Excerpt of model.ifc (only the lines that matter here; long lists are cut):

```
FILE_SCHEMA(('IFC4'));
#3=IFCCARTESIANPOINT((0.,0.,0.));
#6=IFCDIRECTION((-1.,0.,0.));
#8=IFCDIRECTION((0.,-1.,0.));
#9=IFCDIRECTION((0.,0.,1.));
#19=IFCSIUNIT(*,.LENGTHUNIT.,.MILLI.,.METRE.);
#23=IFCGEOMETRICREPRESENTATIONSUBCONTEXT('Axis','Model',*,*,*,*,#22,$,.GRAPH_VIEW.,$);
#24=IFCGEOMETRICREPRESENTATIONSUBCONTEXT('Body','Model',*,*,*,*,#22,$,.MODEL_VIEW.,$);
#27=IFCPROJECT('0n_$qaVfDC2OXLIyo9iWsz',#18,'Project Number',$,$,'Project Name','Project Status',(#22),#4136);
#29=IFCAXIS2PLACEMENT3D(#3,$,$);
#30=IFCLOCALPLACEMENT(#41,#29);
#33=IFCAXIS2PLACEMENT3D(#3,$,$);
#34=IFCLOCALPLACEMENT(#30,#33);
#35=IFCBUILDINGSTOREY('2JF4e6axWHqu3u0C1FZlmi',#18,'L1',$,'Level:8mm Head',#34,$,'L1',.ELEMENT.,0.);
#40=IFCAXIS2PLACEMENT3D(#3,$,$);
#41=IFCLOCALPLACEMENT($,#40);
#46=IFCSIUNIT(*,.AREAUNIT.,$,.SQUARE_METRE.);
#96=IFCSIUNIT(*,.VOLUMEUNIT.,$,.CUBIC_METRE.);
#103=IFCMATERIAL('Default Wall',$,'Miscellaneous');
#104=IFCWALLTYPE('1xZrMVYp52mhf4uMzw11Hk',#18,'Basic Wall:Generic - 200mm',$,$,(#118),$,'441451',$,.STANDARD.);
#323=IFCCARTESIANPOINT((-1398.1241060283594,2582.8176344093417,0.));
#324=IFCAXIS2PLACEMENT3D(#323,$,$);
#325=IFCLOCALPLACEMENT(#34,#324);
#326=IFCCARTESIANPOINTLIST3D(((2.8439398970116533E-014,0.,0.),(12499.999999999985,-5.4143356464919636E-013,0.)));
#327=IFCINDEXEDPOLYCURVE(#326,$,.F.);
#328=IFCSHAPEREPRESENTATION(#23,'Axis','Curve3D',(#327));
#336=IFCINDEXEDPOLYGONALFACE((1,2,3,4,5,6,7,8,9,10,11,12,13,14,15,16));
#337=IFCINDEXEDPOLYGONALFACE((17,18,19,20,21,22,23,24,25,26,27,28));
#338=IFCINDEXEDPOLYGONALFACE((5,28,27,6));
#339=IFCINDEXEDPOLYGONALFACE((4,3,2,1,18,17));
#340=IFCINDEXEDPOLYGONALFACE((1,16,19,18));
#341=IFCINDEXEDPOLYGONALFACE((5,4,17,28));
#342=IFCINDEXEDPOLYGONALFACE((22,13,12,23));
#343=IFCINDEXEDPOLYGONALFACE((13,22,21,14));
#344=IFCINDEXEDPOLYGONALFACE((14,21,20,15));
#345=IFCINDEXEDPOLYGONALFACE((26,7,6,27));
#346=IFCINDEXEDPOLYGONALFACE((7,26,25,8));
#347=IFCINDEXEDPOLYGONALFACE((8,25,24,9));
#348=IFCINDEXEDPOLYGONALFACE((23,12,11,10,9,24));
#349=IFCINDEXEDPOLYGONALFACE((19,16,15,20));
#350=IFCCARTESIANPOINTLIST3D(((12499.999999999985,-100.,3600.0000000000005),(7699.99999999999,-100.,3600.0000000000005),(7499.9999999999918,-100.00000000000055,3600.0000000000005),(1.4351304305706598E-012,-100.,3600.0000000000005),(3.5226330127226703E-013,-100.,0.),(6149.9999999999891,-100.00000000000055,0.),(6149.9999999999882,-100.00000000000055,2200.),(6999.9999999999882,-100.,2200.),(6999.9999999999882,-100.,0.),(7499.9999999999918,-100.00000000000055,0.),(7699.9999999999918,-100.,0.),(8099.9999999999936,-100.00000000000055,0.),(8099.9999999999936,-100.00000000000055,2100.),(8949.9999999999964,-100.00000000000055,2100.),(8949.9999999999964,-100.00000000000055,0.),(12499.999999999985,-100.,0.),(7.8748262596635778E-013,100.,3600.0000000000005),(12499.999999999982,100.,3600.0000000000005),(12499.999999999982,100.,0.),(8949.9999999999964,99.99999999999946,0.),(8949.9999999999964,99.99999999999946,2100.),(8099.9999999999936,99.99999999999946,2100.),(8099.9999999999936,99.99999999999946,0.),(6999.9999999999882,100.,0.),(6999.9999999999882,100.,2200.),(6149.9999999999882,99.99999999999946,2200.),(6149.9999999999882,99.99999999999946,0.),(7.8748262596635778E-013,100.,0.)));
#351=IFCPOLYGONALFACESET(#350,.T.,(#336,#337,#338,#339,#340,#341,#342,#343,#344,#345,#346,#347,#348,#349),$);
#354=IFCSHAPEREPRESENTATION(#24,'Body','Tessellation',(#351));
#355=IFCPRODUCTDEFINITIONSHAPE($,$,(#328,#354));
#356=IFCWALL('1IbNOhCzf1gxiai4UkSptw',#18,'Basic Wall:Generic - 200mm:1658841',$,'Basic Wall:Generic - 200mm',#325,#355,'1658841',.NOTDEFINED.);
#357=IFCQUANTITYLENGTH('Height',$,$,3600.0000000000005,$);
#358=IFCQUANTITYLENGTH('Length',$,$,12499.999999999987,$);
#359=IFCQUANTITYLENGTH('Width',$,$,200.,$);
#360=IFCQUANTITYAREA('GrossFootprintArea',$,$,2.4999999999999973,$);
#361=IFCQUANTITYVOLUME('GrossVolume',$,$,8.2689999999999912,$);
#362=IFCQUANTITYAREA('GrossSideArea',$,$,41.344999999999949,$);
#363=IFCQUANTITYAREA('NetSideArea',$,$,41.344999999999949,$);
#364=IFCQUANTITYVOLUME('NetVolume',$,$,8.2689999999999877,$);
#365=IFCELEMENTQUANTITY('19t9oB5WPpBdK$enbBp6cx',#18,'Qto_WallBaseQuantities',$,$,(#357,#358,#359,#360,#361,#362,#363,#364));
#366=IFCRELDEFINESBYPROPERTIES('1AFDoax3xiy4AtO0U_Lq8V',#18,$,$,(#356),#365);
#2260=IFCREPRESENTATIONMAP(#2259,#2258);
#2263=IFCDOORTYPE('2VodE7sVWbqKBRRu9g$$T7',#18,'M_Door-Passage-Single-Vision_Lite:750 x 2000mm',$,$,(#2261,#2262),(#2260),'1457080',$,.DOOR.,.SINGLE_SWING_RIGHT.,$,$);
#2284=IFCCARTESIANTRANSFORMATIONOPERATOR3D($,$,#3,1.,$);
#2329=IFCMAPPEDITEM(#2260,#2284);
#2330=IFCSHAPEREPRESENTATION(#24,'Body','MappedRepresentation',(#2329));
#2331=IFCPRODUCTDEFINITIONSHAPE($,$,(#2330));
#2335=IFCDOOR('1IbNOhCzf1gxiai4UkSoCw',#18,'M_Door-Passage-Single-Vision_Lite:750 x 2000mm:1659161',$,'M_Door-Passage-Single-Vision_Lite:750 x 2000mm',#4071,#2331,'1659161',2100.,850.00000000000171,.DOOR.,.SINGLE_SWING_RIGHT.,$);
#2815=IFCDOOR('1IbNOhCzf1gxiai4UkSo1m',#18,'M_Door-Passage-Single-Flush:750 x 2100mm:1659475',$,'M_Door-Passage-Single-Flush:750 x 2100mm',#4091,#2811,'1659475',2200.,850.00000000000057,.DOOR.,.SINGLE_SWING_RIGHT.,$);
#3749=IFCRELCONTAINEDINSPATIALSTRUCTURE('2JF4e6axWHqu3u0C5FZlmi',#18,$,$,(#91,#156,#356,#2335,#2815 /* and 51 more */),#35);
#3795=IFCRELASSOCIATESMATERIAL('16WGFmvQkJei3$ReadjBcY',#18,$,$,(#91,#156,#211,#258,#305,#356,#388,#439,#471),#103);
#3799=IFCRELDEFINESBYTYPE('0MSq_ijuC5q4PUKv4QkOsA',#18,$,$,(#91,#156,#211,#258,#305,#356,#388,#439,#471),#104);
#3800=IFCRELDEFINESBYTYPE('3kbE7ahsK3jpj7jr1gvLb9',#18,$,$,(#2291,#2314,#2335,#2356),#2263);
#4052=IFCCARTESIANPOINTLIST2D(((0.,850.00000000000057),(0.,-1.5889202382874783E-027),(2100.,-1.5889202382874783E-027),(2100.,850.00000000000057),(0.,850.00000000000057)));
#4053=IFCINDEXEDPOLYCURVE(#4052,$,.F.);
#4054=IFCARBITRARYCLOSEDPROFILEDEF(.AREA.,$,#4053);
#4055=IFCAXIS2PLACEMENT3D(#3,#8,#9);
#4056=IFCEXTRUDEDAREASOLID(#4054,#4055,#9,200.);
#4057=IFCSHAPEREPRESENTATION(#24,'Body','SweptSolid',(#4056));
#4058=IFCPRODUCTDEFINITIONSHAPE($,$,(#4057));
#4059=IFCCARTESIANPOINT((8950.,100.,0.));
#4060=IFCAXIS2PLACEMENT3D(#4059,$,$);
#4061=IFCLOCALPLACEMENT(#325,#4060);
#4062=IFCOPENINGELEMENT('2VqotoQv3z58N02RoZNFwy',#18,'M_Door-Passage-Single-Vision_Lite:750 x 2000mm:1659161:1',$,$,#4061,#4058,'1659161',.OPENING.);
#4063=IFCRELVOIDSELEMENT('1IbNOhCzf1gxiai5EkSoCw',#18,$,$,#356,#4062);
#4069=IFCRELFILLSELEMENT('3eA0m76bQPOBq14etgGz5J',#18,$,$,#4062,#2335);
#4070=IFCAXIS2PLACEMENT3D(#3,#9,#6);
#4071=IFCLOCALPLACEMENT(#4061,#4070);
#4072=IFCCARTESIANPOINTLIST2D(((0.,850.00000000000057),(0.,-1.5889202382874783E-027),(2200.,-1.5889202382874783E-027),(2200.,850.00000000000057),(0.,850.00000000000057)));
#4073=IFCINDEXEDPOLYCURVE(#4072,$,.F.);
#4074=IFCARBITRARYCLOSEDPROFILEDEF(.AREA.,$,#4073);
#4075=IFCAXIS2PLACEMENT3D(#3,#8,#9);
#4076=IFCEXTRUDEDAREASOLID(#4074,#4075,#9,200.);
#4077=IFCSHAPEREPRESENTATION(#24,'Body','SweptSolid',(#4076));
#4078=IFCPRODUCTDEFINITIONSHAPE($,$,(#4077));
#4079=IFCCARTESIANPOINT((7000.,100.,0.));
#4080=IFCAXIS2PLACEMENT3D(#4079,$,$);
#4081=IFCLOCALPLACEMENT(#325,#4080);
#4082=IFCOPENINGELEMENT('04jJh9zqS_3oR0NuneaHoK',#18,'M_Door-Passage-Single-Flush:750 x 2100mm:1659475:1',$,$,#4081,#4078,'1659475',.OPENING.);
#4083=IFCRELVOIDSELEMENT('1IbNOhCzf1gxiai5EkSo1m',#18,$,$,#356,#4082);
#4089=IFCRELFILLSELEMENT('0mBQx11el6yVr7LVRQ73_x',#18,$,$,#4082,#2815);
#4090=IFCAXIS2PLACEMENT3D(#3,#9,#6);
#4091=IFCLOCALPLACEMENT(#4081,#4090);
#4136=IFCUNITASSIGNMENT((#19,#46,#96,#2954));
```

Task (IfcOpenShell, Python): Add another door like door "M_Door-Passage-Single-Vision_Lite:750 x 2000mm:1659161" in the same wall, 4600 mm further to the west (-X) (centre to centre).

```python
import ifcopenshell
import ifcopenshell.api.feature
import ifcopenshell.api.geometry
import ifcopenshell.api.pset
import ifcopenshell.api.root
import ifcopenshell.geom
import ifcopenshell.util.element
import ifcopenshell.util.placement
import ifcopenshell.util.shape
import ifcopenshell.util.unit

model = ifcopenshell.open("model.ifc")
unit_scale = ifcopenshell.util.unit.calculate_unit_scale(model)
area_scale = ifcopenshell.util.unit.calculate_unit_scale(model, "AREAUNIT")
volume_scale = ifcopenshell.util.unit.calculate_unit_scale(model, "VOLUMEUNIT")
settings = ifcopenshell.geom.settings()


def volume(element):
    """Net volume in cubic metres, openings subtracted."""
    shape = ifcopenshell.geom.create_shape(settings, element)
    return ifcopenshell.util.shape.get_volume(shape.geometry)


def reuse_history(source, copy):
    """copy_class also copies each property set's owner history, people and application; keep the originals."""
    for rel in copy.IsDefinedBy:
        if rel.is_a("IfcRelDefinesByProperties") and (history := rel.RelatingPropertyDefinition.OwnerHistory):
            rel.RelatingPropertyDefinition.OwnerHistory = source.OwnerHistory
            ifcopenshell.util.element.remove_deep2(model, history)


door = model.by_id(2335)
opening = door.FillsVoids[0].RelatingOpeningElement
wall = opening.VoidsElements[0].RelatingBuildingElement
before = volume(wall)
shift = ifcopenshell.util.placement.get_local_placement(wall.ObjectPlacement)[:3, 0] * -4.6 / unit_scale

# copy_class copies the void relationship, type, container and properties, but no geometry.
new_opening = ifcopenshell.api.root.copy_class(model, product=opening)
new_opening.Representation = ifcopenshell.util.element.copy_deep(
    model, opening.Representation, exclude=["IfcGeometricRepresentationContext", "IfcRepresentationMap"]
)
new_opening.Name = "M_Door-Passage-Single-Vision_Lite:750 x 2000mm"
new_opening.Tag = None
reuse_history(opening, new_opening)
new_door = ifcopenshell.api.root.copy_class(model, product=door)
new_door.Representation = ifcopenshell.util.element.copy_deep(
    model, door.Representation, exclude=["IfcGeometricRepresentationContext", "IfcRepresentationMap"]
)
new_door.Name = "M_Door-Passage-Single-Vision_Lite:750 x 2000mm"
new_door.Tag = None
reuse_history(door, new_door)
ifcopenshell.api.feature.add_filling(model, opening=new_opening, element=new_door)

for old, new in ((opening, new_opening), (door, new_door)):
    matrix = ifcopenshell.util.placement.get_local_placement(old.ObjectPlacement)
    matrix[:3, 3] += shift
    ifcopenshell.api.geometry.edit_object_placement(model, product=new, matrix=matrix, is_si=False)

after = volume(wall)
thickness = 0.2  # wall thickness in metres

# Update the wall's stored quantities.
qto = model.by_id(ifcopenshell.util.element.get_pset(wall, "Qto_WallBaseQuantities", should_inherit=False)["id"])
ifcopenshell.api.pset.edit_qto(model, qto=qto, properties={
    "NetSideArea": after / thickness / area_scale,
    "NetVolume": after / volume_scale,
})

print(f"wall volume {before:.3f} -> {after:.3f} m3")

model.write("model_v2.ifc")
```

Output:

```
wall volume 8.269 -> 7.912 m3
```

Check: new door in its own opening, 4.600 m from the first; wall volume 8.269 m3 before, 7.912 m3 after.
